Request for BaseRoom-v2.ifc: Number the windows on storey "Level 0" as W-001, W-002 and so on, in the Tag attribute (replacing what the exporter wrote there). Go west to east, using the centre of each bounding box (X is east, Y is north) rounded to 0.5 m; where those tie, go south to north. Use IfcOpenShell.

First a look at what the model holds.

```python
import ifcopenshell
import ifcopenshell.util.element
import ifcopenshell.util.placement

model = ifcopenshell.open("BaseRoom-v2.ifc")
print(model.schema)
storey = next(s for s in model.by_type("IfcBuildingStorey") if s.Name == "Level 0")
windows = [e for e in ifcopenshell.util.element.get_decomposition(storey) if e.is_a("IfcWindow")]
for e in sorted(windows, key=lambda e: e.id()):
    origin = ifcopenshell.util.placement.get_local_placement(e.ObjectPlacement)[:3, 3]
    print(e.id(), e.Tag, e.Name, origin.round(2) + 0.0, sep=" | ")
```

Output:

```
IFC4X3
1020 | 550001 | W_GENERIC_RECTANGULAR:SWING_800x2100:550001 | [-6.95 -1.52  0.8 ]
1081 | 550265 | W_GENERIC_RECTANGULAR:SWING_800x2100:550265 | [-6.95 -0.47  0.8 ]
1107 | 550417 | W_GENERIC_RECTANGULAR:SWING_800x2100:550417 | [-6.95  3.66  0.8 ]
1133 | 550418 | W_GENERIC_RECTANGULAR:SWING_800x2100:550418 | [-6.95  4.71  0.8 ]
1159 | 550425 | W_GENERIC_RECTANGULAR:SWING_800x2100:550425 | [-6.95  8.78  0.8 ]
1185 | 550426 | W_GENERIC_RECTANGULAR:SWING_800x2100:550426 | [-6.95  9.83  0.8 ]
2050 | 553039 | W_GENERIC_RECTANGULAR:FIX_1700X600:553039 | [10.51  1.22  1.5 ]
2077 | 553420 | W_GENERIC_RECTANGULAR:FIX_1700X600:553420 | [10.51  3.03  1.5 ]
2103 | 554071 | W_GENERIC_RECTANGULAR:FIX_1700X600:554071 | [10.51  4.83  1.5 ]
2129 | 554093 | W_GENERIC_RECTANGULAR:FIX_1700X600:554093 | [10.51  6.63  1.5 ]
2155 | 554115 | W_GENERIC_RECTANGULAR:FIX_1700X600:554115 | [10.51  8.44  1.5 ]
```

```python
import ifcopenshell
import ifcopenshell.geom
import ifcopenshell.util.element
import ifcopenshell.util.shape

model = ifcopenshell.open("BaseRoom-v2.ifc")
settings = ifcopenshell.geom.settings()
settings.set("use-world-coords", True)


def centre(element):
    shape = ifcopenshell.geom.create_shape(settings, element)
    return ifcopenshell.util.shape.get_bbox_centroid(shape.geometry)


storey = next(s for s in model.by_type("IfcBuildingStorey") if s.Name == "Level 0")
windows = [e for e in ifcopenshell.util.element.get_decomposition(storey) if e.is_a("IfcWindow")]

# Insertion points can sit at a corner or the storey origin, so sort by the geometry (in metres).
centres = {e: centre(e) for e in windows}
windows.sort(key=lambda e: (round(centres[e][0] / 0.5), centres[e][1]))

for i, e in enumerate(windows, start=1):
    number = f"W-0{i:02d}"
    e.Tag = number
    print(e.id(), number)

model.write("BaseRoom-v2_rev.ifc")
```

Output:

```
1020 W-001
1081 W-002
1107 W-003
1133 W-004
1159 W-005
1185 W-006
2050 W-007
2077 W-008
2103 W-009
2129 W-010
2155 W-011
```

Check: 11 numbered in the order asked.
